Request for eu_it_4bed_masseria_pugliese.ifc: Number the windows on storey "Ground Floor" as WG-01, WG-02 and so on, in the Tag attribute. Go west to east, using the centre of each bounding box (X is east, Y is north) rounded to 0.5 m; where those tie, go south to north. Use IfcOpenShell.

First a look at what the model holds.

```python
import ifcopenshell
import ifcopenshell.util.element
import ifcopenshell.util.placement

model = ifcopenshell.open("eu_it_4bed_masseria_pugliese.ifc")
print(model.schema)
storey = next(s for s in model.by_type("IfcBuildingStorey") if s.Name == "Ground Floor")
windows = [e for e in ifcopenshell.util.element.get_decomposition(storey) if e.is_a("IfcWindow")]
for e in sorted(windows, key=lambda e: e.id()):
    origin = ifcopenshell.util.placement.get_local_placement(e.ObjectPlacement)[:3, 3]
    print(e.id(), e.Tag, e.Name, origin.round(2) + 0.0, sep=" | ")
```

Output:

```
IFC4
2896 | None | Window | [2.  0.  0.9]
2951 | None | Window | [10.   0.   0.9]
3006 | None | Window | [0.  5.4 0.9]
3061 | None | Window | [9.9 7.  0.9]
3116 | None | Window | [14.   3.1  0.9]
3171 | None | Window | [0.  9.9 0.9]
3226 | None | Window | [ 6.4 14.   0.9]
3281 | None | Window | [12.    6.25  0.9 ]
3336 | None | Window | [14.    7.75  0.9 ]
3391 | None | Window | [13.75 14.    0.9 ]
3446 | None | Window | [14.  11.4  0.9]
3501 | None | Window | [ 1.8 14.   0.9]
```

```python
import ifcopenshell
import ifcopenshell.geom
import ifcopenshell.util.element
import ifcopenshell.util.shape

model = ifcopenshell.open("eu_it_4bed_masseria_pugliese.ifc")
settings = ifcopenshell.geom.settings()
settings.set("use-world-coords", True)


def centre(element):
    shape = ifcopenshell.geom.create_shape(settings, element)
    return ifcopenshell.util.shape.get_bbox_centroid(shape.geometry)


storey = next(s for s in model.by_type("IfcBuildingStorey") if s.Name == "Ground Floor")
windows = [e for e in ifcopenshell.util.element.get_decomposition(storey) if e.is_a("IfcWindow")]

# Insertion points can sit at a corner or the storey origin, so sort by the geometry (in metres).
centres = {e: centre(e) for e in windows}
windows.sort(key=lambda e: (round(centres[e][0] / 0.5), centres[e][1]))

for i, e in enumerate(windows, start=1):
    number = f"WG-{i:02d}"
    e.Tag = number
    print(e.id(), number)

model.write("eu_it_4bed_masseria_pugliese-out.ifc")
```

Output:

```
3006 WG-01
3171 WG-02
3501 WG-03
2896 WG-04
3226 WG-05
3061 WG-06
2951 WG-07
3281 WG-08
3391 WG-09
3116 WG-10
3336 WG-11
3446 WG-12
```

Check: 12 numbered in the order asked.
